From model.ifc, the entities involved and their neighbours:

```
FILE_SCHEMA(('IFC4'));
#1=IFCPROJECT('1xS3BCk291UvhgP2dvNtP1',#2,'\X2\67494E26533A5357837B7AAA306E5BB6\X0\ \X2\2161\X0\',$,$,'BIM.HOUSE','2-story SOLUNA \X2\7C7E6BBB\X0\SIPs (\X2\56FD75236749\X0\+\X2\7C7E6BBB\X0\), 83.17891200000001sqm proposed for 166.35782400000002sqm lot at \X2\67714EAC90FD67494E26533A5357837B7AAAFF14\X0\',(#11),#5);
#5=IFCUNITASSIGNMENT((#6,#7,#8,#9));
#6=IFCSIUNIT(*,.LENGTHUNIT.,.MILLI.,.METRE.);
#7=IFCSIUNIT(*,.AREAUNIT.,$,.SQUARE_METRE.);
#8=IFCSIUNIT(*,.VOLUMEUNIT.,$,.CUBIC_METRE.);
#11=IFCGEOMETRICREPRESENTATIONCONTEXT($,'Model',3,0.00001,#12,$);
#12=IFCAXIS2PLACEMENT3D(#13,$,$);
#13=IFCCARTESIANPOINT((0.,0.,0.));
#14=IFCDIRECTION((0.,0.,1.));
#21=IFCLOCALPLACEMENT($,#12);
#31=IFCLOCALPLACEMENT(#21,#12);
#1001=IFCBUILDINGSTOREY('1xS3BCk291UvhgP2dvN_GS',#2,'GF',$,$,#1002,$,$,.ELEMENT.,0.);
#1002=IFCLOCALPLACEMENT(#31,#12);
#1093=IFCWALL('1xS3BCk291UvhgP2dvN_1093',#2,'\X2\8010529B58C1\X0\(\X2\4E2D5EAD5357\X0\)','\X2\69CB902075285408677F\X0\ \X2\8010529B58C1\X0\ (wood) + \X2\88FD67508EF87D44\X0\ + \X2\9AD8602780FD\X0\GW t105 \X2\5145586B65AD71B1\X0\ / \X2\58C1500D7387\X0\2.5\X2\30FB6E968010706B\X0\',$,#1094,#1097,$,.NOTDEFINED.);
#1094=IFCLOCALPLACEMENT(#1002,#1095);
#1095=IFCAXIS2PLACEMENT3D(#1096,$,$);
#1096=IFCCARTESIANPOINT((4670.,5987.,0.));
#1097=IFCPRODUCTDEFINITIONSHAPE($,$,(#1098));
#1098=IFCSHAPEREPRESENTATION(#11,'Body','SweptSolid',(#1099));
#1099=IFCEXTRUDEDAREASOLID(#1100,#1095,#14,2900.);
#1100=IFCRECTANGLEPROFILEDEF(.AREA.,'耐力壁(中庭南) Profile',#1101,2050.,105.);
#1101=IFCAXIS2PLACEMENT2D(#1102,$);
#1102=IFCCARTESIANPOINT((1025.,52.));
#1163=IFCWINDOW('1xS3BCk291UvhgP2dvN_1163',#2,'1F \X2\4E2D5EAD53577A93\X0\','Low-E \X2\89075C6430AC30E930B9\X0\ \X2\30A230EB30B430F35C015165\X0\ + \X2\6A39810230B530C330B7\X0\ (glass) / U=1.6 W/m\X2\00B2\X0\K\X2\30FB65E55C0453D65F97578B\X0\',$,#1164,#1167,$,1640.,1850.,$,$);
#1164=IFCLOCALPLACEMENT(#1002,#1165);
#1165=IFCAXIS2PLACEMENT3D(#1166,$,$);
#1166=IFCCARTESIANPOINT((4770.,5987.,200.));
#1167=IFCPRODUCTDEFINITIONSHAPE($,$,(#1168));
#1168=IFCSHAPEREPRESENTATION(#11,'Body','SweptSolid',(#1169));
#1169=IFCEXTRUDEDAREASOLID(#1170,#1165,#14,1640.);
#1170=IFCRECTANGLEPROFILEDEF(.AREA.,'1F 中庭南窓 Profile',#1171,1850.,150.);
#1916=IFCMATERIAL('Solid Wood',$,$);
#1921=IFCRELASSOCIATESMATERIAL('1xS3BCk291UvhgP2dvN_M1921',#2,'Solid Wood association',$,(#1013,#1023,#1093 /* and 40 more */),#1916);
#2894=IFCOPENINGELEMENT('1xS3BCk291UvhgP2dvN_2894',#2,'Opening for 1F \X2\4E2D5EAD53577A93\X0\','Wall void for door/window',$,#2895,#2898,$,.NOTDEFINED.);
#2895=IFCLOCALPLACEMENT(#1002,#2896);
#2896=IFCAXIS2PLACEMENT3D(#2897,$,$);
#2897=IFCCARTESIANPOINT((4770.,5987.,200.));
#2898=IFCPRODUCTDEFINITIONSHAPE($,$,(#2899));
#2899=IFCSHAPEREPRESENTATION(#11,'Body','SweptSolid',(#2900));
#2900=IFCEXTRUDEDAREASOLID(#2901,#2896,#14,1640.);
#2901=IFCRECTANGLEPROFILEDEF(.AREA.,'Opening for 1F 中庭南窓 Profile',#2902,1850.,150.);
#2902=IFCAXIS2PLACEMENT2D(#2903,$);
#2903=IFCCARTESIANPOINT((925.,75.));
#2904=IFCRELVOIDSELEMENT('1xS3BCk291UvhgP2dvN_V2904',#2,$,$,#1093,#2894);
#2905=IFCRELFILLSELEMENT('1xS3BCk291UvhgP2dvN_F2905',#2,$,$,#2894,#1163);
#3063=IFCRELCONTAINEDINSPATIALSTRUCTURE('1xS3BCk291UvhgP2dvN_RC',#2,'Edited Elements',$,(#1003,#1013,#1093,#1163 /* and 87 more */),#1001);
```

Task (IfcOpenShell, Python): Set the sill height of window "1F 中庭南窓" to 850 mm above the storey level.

```python
import numpy as np
import ifcopenshell
import ifcopenshell.api.geometry
import ifcopenshell.geom
import ifcopenshell.util.element
import ifcopenshell.util.placement
import ifcopenshell.util.shape
import ifcopenshell.util.unit

model = ifcopenshell.open("model.ifc")
unit_scale = ifcopenshell.util.unit.calculate_unit_scale(model)

window = model.by_guid("1xS3BCk291UvhgP2dvN_1163")
opening = window.FillsVoids[0].RelatingOpeningElement
storey = ifcopenshell.util.element.get_container(window, ifc_class="IfcBuildingStorey")
level = ifcopenshell.util.placement.get_local_placement(storey.ObjectPlacement)[2, 3]

# The opening's origin need not be at the sill, so measure its lowest point.
shape = ifcopenshell.geom.create_shape(ifcopenshell.geom.settings(), opening)
bottom = ifcopenshell.util.shape.get_shape_bottom_elevation(shape, shape.geometry) / unit_scale
dz = level + 850.0 - bottom

shift = np.array([0.0, 0.0, dz])
# The window is not placed relative to its opening, so move both.
for product in (opening, window):
    matrix = ifcopenshell.util.placement.get_local_placement(product.ObjectPlacement)
    matrix[:3, 3] += shift
    ifcopenshell.api.geometry.edit_object_placement(model, product=product, matrix=matrix, is_si=False)

print(f"moved by {dz * unit_scale:+.3f} m")

model.write("model_updated.ifc")
```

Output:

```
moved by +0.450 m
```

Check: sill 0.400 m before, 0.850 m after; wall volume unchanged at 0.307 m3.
